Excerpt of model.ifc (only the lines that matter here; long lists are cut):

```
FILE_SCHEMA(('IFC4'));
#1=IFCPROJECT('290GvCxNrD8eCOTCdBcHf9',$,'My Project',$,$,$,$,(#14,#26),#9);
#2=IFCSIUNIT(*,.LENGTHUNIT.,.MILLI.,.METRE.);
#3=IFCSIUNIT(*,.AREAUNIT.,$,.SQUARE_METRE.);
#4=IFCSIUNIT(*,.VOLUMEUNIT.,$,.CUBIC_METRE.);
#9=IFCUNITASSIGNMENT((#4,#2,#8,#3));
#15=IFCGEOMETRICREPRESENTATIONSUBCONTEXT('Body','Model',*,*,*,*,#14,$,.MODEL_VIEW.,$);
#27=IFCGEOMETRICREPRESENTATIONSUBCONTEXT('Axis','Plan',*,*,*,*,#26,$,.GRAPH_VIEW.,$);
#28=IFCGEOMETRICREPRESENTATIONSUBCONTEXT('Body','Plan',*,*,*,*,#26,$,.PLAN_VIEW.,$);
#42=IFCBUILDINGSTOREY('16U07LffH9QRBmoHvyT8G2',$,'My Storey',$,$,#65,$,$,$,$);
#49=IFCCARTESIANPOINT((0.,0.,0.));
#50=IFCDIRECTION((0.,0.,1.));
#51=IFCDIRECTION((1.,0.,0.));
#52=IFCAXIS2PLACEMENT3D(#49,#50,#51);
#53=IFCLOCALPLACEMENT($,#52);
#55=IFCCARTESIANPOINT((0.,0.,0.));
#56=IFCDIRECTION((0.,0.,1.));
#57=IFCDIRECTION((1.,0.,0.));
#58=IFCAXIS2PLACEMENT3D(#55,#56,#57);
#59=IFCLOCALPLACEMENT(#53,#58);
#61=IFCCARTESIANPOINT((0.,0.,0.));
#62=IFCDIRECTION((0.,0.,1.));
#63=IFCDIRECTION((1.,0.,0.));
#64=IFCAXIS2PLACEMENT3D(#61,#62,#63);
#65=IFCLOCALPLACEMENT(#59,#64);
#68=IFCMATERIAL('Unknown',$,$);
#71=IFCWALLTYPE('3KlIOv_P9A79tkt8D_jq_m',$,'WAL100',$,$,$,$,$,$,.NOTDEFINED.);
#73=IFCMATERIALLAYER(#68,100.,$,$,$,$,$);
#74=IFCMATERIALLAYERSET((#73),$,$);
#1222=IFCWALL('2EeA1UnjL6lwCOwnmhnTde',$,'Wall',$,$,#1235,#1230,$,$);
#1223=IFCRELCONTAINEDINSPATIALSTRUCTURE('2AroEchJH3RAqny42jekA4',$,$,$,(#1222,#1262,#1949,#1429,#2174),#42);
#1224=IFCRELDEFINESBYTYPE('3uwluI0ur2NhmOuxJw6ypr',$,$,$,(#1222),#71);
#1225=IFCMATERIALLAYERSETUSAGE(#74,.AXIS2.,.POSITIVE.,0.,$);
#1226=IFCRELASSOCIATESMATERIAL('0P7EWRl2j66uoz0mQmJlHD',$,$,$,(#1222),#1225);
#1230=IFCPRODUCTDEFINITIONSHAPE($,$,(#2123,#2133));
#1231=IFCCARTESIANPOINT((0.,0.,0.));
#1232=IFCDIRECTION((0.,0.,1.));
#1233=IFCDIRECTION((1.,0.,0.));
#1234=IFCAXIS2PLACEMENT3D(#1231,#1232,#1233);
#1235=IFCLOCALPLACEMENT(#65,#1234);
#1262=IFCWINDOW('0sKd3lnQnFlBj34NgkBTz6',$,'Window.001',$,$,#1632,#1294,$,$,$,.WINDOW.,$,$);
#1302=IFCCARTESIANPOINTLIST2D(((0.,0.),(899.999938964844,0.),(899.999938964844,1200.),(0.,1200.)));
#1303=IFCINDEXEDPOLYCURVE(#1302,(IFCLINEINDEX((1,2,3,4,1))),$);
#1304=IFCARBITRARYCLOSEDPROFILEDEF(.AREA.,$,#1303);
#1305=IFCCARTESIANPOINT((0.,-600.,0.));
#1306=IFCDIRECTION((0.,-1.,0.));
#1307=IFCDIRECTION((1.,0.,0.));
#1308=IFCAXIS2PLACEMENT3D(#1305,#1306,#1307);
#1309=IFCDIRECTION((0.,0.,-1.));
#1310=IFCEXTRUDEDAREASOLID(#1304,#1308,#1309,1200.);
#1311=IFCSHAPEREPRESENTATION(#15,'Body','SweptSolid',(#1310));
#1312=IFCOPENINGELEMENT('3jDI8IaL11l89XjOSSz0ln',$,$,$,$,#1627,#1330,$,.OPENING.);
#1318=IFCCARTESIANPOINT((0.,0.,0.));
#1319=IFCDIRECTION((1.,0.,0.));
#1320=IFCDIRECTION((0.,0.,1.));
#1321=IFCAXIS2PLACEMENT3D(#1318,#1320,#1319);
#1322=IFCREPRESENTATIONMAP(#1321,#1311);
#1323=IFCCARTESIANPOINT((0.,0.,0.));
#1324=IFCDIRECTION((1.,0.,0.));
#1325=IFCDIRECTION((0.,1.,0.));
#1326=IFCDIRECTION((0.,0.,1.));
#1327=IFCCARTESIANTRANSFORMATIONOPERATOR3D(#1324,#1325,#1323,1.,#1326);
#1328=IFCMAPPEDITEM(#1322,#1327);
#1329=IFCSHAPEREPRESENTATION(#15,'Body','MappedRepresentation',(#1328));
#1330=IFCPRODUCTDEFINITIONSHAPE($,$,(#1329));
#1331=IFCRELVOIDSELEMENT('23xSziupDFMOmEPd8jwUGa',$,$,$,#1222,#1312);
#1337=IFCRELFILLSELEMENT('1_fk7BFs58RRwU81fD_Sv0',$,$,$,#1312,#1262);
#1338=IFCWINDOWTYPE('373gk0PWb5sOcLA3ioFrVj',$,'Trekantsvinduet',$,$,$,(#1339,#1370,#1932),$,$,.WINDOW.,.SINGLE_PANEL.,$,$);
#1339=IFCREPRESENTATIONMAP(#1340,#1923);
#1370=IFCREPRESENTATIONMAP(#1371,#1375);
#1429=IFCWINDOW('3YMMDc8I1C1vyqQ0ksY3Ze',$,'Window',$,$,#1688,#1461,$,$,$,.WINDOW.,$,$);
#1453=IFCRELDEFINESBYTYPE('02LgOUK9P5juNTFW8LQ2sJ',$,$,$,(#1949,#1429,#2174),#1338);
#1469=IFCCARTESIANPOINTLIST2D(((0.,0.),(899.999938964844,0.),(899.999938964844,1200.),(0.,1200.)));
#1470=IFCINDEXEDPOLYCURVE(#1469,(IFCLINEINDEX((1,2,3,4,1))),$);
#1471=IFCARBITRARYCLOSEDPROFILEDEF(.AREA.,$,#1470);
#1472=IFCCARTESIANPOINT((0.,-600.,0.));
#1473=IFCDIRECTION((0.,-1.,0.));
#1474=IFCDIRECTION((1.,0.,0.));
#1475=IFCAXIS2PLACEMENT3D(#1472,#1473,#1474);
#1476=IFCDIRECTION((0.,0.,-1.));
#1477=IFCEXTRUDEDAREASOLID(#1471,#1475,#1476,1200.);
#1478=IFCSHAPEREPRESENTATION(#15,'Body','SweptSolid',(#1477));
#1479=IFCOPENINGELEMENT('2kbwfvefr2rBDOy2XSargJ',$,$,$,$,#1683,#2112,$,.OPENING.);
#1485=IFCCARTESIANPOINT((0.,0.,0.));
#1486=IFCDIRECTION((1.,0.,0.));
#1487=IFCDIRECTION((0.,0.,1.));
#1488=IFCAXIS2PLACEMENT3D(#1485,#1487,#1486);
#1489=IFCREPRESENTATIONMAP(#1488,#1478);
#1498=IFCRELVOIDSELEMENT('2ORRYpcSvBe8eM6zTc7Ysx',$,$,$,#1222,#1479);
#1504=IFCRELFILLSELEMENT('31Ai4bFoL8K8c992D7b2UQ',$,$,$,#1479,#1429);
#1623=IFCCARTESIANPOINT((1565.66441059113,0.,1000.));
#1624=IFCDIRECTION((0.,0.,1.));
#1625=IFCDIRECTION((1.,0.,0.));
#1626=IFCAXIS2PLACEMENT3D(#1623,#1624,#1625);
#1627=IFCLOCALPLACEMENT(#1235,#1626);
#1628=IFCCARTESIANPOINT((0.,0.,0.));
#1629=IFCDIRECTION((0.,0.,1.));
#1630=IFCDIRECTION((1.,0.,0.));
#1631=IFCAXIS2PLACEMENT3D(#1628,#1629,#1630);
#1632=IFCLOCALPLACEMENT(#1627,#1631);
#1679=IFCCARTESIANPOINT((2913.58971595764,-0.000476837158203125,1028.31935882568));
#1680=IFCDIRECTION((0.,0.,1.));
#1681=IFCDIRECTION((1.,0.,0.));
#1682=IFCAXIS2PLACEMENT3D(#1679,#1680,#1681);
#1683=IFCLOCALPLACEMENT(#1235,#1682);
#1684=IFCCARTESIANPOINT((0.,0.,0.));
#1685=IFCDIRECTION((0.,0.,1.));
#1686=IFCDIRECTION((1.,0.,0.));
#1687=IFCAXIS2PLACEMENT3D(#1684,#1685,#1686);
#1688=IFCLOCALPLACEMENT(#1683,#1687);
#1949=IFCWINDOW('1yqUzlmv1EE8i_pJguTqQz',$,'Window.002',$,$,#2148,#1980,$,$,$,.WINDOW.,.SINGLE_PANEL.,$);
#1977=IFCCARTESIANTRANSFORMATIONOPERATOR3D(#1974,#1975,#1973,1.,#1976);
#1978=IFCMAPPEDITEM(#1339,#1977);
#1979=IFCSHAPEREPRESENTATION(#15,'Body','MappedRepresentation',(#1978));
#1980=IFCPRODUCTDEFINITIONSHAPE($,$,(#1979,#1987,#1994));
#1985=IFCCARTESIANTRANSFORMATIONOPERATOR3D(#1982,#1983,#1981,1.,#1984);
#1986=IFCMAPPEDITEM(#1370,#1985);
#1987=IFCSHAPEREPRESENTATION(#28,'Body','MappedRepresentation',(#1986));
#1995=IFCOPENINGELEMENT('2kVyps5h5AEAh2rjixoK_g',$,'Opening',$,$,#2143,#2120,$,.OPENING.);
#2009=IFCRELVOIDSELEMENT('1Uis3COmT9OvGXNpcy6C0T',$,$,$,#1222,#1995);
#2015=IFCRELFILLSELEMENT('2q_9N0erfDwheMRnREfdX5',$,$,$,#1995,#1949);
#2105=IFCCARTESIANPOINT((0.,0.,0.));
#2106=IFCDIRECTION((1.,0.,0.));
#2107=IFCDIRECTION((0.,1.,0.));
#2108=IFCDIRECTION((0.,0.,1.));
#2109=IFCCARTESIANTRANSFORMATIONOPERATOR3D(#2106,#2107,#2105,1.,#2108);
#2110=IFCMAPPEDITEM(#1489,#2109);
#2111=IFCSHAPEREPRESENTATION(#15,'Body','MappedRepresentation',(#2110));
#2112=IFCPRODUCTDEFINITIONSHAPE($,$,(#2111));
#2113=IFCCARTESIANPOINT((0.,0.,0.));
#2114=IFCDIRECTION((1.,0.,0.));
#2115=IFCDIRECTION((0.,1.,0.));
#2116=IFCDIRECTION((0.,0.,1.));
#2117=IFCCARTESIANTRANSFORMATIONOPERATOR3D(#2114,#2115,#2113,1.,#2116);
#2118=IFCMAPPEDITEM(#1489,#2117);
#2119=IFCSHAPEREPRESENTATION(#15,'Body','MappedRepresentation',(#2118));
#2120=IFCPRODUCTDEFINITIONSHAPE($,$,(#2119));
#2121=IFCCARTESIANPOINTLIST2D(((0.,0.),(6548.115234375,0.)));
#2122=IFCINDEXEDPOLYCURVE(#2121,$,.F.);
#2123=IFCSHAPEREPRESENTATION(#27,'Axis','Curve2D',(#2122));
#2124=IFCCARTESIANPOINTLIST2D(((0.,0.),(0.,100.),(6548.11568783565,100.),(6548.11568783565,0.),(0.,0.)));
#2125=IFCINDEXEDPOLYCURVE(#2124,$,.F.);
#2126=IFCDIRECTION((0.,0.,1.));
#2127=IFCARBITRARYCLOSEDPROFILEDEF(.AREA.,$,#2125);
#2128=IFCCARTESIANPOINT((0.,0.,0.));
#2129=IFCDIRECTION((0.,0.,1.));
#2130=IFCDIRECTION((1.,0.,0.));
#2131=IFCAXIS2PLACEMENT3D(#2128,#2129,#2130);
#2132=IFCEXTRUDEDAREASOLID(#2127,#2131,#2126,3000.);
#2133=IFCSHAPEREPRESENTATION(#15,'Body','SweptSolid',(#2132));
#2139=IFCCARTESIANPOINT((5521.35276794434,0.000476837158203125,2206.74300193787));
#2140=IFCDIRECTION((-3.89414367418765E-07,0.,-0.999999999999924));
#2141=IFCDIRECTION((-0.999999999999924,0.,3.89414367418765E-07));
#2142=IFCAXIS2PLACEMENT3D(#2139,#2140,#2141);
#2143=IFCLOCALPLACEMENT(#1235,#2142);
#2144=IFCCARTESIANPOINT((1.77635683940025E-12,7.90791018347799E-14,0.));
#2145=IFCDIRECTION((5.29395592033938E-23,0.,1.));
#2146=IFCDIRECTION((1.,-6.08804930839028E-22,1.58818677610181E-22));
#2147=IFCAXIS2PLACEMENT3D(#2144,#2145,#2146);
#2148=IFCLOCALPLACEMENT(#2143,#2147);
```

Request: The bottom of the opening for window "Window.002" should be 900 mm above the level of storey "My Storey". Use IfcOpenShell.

```python
import numpy as np
import ifcopenshell
import ifcopenshell.api.geometry
import ifcopenshell.geom
import ifcopenshell.util.element
import ifcopenshell.util.placement
import ifcopenshell.util.shape
import ifcopenshell.util.unit

model = ifcopenshell.open("model.ifc")
unit_scale = ifcopenshell.util.unit.calculate_unit_scale(model)

window = model.by_guid("1yqUzlmv1EE8i_pJguTqQz")
opening = window.FillsVoids[0].RelatingOpeningElement
storey = ifcopenshell.util.element.get_container(window, ifc_class="IfcBuildingStorey")
level = ifcopenshell.util.placement.get_local_placement(storey.ObjectPlacement)[2, 3]

# The opening's origin need not be at the sill, so measure its lowest point.
shape = ifcopenshell.geom.create_shape(ifcopenshell.geom.settings(), opening)
bottom = ifcopenshell.util.shape.get_shape_bottom_elevation(shape, shape.geometry) / unit_scale
dz = level + 900.0 - bottom

shift = np.array([0.0, 0.0, dz])
# The window is placed relative to its opening, so it follows when the opening moves.
matrix = ifcopenshell.util.placement.get_local_placement(opening.ObjectPlacement)
matrix[:3, 3] += shift
ifcopenshell.api.geometry.edit_object_placement(
    model, product=opening, matrix=matrix, is_si=False, should_transform_children=True
)

print(f"moved by {dz * unit_scale:+.3f} m")

model.write("model-out.ifc")
```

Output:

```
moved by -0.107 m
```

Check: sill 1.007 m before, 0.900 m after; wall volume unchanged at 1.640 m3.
